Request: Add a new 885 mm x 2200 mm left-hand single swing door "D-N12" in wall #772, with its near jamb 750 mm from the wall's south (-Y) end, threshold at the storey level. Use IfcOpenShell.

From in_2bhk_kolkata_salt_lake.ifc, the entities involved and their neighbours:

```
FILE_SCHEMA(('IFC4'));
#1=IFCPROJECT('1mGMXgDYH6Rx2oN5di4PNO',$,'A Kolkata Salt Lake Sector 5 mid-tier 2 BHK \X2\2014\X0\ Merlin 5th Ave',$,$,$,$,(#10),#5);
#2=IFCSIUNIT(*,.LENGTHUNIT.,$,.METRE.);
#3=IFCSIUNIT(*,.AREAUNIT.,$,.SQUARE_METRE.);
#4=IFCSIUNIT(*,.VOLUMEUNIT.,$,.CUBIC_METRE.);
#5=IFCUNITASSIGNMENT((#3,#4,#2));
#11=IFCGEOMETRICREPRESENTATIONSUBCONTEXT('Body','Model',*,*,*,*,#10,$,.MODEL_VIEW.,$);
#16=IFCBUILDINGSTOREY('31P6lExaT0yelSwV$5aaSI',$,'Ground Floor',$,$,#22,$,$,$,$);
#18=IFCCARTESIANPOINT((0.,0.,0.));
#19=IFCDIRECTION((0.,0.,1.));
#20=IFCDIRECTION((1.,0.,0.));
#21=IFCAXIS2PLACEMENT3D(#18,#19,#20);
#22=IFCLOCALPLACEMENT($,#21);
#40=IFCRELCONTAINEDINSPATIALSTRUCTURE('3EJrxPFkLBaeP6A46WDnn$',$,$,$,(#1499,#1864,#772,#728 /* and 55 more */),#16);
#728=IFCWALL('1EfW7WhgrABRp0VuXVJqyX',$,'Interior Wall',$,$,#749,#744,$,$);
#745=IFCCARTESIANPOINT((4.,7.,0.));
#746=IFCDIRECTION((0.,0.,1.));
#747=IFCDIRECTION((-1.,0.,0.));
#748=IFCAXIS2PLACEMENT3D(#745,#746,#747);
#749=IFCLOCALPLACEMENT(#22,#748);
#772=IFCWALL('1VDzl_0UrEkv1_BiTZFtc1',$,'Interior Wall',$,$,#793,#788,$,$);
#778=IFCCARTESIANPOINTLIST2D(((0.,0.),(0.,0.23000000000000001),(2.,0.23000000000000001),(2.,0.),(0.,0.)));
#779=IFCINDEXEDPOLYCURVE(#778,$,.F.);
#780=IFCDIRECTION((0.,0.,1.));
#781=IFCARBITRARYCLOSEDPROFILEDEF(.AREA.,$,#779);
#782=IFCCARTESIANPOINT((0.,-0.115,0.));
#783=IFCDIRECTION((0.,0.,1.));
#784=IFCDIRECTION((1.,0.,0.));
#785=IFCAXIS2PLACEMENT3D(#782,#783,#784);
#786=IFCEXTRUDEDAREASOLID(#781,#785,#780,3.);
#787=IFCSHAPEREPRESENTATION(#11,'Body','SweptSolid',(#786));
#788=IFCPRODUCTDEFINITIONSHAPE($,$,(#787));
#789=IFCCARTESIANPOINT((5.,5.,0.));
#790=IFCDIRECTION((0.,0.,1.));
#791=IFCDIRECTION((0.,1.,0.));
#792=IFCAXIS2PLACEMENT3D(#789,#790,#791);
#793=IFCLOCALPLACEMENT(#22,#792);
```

```python
import numpy as np
import ifcopenshell
import ifcopenshell.api.feature
import ifcopenshell.api.geometry
import ifcopenshell.api.root
import ifcopenshell.api.spatial
import ifcopenshell.geom
import ifcopenshell.util.element
import ifcopenshell.util.placement
import ifcopenshell.util.representation
import ifcopenshell.util.shape
import ifcopenshell.util.unit

model = ifcopenshell.open("in_2bhk_kolkata_salt_lake.ifc")
unit_scale = ifcopenshell.util.unit.calculate_unit_scale(model)
settings = ifcopenshell.geom.settings()


def volume(element):
    """Net volume in cubic metres, openings subtracted."""
    shape = ifcopenshell.geom.create_shape(settings, element)
    return ifcopenshell.util.shape.get_volume(shape.geometry)


wall = model.by_id(772)
storey = ifcopenshell.util.element.get_container(wall, ifc_class="IfcBuildingStorey")
context = ifcopenshell.util.representation.get_context(model, "Model", "Body", "MODEL_VIEW")
before = volume(wall)

width, height, from_end, sill = 0.885, 2.2, 0.75, 0.0  # metres

# The wall runs along its own X axis, and the end named is its -X end.
wall_shape = ifcopenshell.geom.create_shape(settings, wall)
x, y, z = ifcopenshell.util.shape.get_vertices(wall_shape.geometry).T
start = x.min() + from_end
face, thickness = float(y.min()), float(y.max() - y.min())
wall_matrix = ifcopenshell.util.placement.get_local_placement(wall.ObjectPlacement)
level = ifcopenshell.util.placement.get_local_placement(storey.ObjectPlacement)[2, 3]


def in_wall(x, y):
    """Placement at x, y metres in the wall's axes, at sill height."""
    matrix = wall_matrix.copy()
    matrix[:, 3] = wall_matrix @ np.array([x / unit_scale, y / unit_scale, 0.0, 1.0])
    matrix[2, 3] = level + sill / unit_scale
    return matrix


# Opening: a box that overshoots both wall faces by 50 mm.
opening = ifcopenshell.api.root.create_entity(model, ifc_class="IfcOpeningElement", predefined_type="OPENING")
box = ifcopenshell.api.geometry.add_wall_representation(
    model, context=context, length=width, height=height, thickness=thickness + 0.1
)
ifcopenshell.api.geometry.assign_representation(model, product=opening, representation=box)
ifcopenshell.api.geometry.edit_object_placement(model, product=opening, matrix=in_wall(start, face - 0.05), is_si=False)
ifcopenshell.api.feature.add_feature(model, feature=opening, element=wall)

door = ifcopenshell.api.root.create_entity(model, ifc_class="IfcDoor", name="D-N12", predefined_type="DOOR")
door.OverallWidth, door.OverallHeight = width / unit_scale, height / unit_scale
door.OperationType = "SINGLE_SWING_LEFT"
body = ifcopenshell.api.geometry.add_door_representation(
    model,
    context=context,
    overall_width=door.OverallWidth,
    overall_height=door.OverallHeight,
    operation_type="SINGLE_SWING_LEFT",
    lining_properties={"LiningDepth": thickness / unit_scale, "ThresholdDepth": thickness / unit_scale},
)
ifcopenshell.api.geometry.assign_representation(model, product=door, representation=body)
ifcopenshell.api.spatial.assign_container(model, products=[door], relating_structure=storey)
ifcopenshell.api.feature.add_filling(model, opening=opening, element=door)

# The lining spans the wall, so the door starts at the wall face.
ifcopenshell.api.geometry.edit_object_placement(model, product=door, matrix=in_wall(start, face), is_si=False)

after = volume(wall)

print(f"wall volume {before:.3f} -> {after:.3f} m3")

model.write("in_2bhk_kolkata_salt_lake_edited.ifc")
```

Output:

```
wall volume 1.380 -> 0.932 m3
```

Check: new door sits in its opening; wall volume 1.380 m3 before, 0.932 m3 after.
